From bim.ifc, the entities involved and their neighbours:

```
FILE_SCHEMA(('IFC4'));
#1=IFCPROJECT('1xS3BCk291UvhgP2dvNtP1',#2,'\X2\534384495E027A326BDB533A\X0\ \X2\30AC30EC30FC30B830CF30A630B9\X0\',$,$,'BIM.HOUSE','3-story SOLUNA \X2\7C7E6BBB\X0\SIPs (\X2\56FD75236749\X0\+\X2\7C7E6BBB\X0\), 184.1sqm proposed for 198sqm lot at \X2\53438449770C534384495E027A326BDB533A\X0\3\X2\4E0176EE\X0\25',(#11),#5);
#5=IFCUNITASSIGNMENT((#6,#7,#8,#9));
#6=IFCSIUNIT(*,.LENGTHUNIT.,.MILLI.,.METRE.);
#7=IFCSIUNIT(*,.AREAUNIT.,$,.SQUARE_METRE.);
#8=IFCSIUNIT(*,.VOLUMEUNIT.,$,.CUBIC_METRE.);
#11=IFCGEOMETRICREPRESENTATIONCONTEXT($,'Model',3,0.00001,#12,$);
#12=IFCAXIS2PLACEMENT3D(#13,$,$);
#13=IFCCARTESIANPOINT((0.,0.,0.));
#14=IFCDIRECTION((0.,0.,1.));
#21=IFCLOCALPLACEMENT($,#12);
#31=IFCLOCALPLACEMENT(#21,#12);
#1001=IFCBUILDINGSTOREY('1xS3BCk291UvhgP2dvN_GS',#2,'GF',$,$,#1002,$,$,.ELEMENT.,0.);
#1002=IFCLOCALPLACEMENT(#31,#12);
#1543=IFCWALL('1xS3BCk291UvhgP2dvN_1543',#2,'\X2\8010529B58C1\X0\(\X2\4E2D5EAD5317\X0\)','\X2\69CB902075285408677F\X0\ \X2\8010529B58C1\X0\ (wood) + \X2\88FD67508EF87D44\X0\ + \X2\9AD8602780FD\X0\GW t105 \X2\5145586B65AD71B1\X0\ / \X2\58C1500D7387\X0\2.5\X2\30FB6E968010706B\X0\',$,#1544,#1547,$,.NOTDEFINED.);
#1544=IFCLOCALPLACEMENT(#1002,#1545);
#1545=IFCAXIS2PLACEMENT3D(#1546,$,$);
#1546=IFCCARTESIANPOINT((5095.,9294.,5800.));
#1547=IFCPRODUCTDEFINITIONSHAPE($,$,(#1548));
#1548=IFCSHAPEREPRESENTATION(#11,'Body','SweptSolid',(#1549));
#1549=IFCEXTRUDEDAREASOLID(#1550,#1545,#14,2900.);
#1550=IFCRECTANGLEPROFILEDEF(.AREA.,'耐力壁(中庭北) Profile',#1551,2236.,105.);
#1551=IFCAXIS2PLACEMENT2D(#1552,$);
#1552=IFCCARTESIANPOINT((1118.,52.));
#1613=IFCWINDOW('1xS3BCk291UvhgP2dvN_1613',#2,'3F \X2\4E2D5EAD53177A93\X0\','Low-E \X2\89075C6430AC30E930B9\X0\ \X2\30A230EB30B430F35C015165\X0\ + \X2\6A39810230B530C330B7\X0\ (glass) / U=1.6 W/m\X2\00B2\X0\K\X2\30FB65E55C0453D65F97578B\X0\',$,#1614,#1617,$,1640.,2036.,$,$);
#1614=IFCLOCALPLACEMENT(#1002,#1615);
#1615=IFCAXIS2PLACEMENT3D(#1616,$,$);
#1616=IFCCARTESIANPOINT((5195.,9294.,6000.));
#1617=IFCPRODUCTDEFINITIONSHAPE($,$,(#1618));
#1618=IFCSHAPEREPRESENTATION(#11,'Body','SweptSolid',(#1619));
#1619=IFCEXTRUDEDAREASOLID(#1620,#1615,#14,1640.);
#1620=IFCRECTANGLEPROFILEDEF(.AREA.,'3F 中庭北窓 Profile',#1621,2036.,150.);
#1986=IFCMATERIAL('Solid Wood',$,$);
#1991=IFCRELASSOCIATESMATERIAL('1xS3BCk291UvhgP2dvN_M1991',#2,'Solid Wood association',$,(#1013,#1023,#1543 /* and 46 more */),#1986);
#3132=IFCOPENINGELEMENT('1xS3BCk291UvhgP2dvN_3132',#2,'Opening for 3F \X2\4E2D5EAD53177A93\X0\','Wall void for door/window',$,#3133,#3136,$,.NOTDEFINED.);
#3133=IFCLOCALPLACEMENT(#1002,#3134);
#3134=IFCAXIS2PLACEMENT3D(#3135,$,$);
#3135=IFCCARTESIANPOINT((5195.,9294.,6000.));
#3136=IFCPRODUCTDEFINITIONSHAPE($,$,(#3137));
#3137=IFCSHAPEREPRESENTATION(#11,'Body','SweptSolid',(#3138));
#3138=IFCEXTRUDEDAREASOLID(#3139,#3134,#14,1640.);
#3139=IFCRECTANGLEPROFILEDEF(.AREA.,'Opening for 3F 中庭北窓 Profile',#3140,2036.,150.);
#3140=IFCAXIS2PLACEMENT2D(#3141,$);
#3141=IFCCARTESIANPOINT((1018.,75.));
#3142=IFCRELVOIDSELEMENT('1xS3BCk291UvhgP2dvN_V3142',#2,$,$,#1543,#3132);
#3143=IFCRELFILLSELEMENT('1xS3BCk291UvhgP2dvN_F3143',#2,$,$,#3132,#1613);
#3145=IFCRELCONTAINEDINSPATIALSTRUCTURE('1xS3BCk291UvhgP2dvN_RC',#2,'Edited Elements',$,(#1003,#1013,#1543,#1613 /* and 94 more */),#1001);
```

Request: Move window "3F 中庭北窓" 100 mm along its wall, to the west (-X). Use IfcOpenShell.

```python
import ifcopenshell
import ifcopenshell.api.geometry
import ifcopenshell.util.placement
import ifcopenshell.util.unit

model = ifcopenshell.open("bim.ifc")
unit_scale = ifcopenshell.util.unit.calculate_unit_scale(model)

window = model.by_id(1613)
opening = window.FillsVoids[0].RelatingOpeningElement
wall = opening.VoidsElements[0].RelatingBuildingElement

wall_matrix = ifcopenshell.util.placement.get_local_placement(wall.ObjectPlacement)
shift = wall_matrix[:3, 0] * -0.1 / unit_scale
before = ifcopenshell.util.placement.get_local_placement(window.ObjectPlacement)[:3, 3].copy()

# The window is not placed relative to its opening, so move both.
for product in (opening, window):
    matrix = ifcopenshell.util.placement.get_local_placement(product.ObjectPlacement)
    matrix[:3, 3] += shift
    ifcopenshell.api.geometry.edit_object_placement(model, product=product, matrix=matrix, is_si=False)

after = ifcopenshell.util.placement.get_local_placement(window.ObjectPlacement)[:3, 3]
print("window moved by", (after - before).round(3) + 0.0)

model.write("bim_updated.ifc")
```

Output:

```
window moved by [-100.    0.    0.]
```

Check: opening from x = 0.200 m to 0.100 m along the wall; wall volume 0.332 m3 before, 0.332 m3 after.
